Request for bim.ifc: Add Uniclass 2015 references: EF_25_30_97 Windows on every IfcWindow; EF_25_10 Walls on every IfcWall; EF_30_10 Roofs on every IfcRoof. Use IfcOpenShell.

First a look at what the model holds.

```python
import ifcopenshell

model = ifcopenshell.open("bim.ifc")
print(model.schema)
print("classifications:", [c.Name for c in model.by_type("IfcClassification")])
for ifc_class in ("IfcDoor", "IfcRoof", "IfcStair", "IfcWall", "IfcWindow"):
    print(ifc_class, len(model.by_type(ifc_class)))
```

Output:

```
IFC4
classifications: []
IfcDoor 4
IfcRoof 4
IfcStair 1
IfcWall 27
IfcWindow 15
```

```python
import ifcopenshell
import ifcopenshell.api.classification

model = ifcopenshell.open("bim.ifc")

system = ifcopenshell.api.classification.add_classification(model, classification="Uniclass 2015")

codes = {
    "IfcWindow": ("EF_25_30_97", "Windows"),
    "IfcWall": ("EF_25_10", "Walls"),
    "IfcRoof": ("EF_30_10", "Roofs"),
}
for ifc_class, (code, name) in codes.items():
    products = model.by_type(ifc_class)
    ifcopenshell.api.classification.add_reference(
        model, products=products, classification=system, identification=code, name=name
    )
    print(code, len(products))

model.write("bim-out.ifc")
```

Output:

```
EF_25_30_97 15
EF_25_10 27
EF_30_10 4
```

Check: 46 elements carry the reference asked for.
